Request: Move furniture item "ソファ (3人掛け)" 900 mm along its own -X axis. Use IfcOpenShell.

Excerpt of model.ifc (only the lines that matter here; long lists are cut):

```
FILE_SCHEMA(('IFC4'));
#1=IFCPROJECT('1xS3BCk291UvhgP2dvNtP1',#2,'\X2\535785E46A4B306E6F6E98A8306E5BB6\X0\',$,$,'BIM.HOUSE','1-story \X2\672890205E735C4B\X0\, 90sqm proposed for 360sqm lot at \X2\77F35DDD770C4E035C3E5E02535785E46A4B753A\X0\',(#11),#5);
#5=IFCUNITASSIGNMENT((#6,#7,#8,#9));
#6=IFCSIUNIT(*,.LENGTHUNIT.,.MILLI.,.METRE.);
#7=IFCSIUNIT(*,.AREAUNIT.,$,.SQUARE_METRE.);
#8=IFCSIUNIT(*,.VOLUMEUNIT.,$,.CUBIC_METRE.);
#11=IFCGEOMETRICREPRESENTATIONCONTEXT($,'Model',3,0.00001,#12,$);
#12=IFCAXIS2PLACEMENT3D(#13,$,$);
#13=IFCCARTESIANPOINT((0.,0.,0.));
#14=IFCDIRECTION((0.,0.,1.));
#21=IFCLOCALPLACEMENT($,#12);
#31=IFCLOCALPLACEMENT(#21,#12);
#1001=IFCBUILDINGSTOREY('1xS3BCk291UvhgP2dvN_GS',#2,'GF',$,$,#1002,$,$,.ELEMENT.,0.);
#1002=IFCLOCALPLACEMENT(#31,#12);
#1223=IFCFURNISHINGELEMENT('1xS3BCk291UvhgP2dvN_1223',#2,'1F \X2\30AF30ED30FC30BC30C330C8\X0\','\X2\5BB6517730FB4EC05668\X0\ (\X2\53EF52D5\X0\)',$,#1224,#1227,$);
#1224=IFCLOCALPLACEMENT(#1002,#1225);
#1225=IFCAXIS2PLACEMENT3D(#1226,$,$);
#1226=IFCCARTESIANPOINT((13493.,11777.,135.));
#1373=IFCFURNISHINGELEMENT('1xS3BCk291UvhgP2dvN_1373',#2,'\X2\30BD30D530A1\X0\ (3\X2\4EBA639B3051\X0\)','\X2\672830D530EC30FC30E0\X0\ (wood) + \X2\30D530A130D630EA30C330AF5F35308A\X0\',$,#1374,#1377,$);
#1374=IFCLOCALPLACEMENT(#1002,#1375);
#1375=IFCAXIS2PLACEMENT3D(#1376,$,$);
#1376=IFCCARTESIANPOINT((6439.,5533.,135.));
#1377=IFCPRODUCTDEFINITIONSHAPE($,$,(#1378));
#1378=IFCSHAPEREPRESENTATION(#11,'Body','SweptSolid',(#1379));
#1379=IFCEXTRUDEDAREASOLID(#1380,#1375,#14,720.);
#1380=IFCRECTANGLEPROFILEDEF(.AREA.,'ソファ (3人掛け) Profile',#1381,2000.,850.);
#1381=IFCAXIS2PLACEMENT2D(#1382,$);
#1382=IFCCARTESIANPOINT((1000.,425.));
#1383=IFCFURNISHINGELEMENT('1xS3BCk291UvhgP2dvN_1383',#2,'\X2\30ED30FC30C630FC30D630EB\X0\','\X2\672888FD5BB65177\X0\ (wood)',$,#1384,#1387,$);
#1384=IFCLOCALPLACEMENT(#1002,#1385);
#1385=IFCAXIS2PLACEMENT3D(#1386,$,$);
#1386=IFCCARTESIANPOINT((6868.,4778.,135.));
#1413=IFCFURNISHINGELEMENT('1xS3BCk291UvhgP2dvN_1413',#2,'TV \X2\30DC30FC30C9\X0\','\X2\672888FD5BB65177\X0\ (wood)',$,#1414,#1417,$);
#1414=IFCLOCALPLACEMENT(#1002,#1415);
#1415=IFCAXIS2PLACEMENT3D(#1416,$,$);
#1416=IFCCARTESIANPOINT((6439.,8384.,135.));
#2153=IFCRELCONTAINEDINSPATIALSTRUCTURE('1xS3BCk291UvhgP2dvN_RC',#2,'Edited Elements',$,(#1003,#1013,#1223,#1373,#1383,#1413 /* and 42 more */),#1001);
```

```python
import ifcopenshell
import ifcopenshell.api.geometry
import ifcopenshell.util.placement
import ifcopenshell.util.unit

model = ifcopenshell.open("model.ifc")
unit_scale = ifcopenshell.util.unit.calculate_unit_scale(model)

item = model.by_id(1373)
matrix = ifcopenshell.util.placement.get_local_placement(item.ObjectPlacement)
matrix[:3, 3] -= matrix[:3, 0] * 0.9 / unit_scale
ifcopenshell.api.geometry.edit_object_placement(model, product=item, matrix=matrix, is_si=False)

print(ifcopenshell.util.placement.get_local_placement(item.ObjectPlacement).round(3) + 0.0)

model.write("model_rev.ifc")
```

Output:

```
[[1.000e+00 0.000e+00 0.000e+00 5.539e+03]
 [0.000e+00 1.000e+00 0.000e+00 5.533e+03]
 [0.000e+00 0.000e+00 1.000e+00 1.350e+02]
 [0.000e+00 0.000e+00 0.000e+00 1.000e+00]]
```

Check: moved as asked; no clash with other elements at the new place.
